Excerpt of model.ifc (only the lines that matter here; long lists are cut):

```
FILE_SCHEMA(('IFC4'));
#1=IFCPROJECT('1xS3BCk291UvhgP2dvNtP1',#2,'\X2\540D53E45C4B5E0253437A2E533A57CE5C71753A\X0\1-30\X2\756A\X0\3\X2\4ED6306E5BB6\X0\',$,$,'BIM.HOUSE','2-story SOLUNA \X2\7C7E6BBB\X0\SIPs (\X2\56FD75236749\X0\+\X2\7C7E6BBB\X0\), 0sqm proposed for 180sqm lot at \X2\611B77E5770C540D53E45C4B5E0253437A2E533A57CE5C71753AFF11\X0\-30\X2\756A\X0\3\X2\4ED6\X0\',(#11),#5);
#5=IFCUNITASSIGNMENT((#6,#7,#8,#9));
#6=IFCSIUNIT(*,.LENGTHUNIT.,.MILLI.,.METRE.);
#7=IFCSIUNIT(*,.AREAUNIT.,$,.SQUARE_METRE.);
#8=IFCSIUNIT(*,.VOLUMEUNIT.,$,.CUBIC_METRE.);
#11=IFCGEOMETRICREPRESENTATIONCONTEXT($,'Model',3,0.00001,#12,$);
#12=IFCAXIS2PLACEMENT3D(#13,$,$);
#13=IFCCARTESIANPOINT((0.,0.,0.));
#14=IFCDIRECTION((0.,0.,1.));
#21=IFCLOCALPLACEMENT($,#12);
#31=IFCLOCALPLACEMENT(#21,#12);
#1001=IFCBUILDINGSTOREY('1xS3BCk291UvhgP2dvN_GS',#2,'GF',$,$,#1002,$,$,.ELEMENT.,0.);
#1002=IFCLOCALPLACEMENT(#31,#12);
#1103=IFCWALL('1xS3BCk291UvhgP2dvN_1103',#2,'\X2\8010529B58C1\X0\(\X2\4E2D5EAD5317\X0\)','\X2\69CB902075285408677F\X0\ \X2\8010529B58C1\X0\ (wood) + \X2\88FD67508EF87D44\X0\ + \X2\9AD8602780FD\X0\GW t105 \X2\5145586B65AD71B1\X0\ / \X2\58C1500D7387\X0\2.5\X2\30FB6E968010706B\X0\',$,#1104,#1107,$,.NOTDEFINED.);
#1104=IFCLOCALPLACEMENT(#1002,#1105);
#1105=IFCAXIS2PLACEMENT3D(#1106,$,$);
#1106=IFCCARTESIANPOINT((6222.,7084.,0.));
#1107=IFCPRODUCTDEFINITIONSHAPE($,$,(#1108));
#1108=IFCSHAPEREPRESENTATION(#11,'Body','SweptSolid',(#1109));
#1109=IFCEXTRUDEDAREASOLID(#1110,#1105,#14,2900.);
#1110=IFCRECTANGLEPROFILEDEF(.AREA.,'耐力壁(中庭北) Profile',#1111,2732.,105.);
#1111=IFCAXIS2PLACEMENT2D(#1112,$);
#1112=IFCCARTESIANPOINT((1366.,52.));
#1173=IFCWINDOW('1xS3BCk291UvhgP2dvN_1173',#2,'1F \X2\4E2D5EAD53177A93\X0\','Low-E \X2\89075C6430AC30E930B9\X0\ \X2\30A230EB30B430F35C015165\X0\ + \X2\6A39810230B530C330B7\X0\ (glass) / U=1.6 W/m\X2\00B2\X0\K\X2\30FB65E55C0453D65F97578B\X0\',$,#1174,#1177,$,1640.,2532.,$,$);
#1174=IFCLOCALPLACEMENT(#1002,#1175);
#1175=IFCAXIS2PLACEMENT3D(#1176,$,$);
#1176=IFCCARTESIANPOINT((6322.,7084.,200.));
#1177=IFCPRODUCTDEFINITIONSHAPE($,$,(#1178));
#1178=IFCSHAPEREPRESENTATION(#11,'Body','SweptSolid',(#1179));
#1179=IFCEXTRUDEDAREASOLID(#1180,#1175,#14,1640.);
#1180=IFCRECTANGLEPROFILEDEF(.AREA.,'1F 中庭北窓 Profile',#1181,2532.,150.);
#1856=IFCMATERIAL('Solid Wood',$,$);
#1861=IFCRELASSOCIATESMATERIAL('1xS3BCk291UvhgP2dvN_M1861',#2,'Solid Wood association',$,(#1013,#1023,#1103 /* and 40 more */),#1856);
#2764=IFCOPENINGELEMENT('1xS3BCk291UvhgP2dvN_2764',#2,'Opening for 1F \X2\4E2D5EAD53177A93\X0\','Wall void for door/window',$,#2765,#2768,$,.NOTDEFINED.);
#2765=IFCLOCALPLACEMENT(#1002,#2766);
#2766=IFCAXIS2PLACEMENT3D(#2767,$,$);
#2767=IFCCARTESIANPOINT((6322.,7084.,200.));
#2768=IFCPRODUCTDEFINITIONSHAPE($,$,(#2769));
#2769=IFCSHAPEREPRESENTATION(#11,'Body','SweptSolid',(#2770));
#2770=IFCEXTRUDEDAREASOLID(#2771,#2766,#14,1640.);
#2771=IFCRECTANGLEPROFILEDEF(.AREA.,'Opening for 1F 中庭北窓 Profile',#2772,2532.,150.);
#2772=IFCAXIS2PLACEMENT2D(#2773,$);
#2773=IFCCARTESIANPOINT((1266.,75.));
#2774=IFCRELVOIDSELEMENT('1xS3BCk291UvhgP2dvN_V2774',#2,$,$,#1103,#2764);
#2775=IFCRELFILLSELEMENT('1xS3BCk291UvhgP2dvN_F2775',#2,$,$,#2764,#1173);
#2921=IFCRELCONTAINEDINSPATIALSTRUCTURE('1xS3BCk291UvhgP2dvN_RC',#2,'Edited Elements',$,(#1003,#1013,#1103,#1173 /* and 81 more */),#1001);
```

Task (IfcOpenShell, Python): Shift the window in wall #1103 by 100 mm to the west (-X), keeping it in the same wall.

```python
import ifcopenshell
import ifcopenshell.api.geometry
import ifcopenshell.util.placement

model = ifcopenshell.open("model.ifc")

window = model.by_id(1173)
opening = window.FillsVoids[0].RelatingOpeningElement
wall = opening.VoidsElements[0].RelatingBuildingElement

wall_matrix = ifcopenshell.util.placement.get_local_placement(wall.ObjectPlacement)
shift = wall_matrix[:3, 0] * -100.0
before = ifcopenshell.util.placement.get_local_placement(window.ObjectPlacement)[:3, 3].copy()

# The window is not placed relative to its opening, so move both.
for product in (opening, window):
    matrix = ifcopenshell.util.placement.get_local_placement(product.ObjectPlacement)
    matrix[:3, 3] += shift
    ifcopenshell.api.geometry.edit_object_placement(model, product=product, matrix=matrix, is_si=False)

after = ifcopenshell.util.placement.get_local_placement(window.ObjectPlacement)[:3, 3]
print("window moved by", (after - before).round(3) + 0.0)

model.write("model-out.ifc")
```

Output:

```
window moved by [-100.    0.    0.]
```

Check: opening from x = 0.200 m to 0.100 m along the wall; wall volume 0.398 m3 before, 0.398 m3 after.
